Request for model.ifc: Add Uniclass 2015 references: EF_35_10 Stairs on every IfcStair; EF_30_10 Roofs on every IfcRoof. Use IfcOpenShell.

First a look at what the model holds.

```python
import ifcopenshell

model = ifcopenshell.open("model.ifc")
print(model.schema)
print("classifications:", [c.Name for c in model.by_type("IfcClassification")])
for ifc_class in ("IfcDoor", "IfcRoof", "IfcStair", "IfcWall", "IfcWindow"):
    print(ifc_class, len(model.by_type(ifc_class)))
```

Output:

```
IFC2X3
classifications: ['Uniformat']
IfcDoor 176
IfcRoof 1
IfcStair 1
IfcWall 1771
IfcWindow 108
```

```python
import ifcopenshell
import ifcopenshell.api.classification

model = ifcopenshell.open("model.ifc")

# IFC2X3 requires Source and Edition and has no link from the project to the system.
system = model.create_entity("IfcClassification", Source="NBS", Edition="2015", Name="Uniclass 2015")

codes = {
    "IfcStair": ("EF_35_10", "Stairs"),
    "IfcRoof": ("EF_30_10", "Roofs"),
}
for ifc_class, (code, name) in codes.items():
    products = model.by_type(ifc_class)
    ifcopenshell.api.classification.add_reference(
        model, products=products, classification=system, identification=code, name=name
    )
    print(code, len(products))

model.write("model-out.ifc")
```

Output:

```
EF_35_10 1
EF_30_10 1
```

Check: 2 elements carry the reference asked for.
